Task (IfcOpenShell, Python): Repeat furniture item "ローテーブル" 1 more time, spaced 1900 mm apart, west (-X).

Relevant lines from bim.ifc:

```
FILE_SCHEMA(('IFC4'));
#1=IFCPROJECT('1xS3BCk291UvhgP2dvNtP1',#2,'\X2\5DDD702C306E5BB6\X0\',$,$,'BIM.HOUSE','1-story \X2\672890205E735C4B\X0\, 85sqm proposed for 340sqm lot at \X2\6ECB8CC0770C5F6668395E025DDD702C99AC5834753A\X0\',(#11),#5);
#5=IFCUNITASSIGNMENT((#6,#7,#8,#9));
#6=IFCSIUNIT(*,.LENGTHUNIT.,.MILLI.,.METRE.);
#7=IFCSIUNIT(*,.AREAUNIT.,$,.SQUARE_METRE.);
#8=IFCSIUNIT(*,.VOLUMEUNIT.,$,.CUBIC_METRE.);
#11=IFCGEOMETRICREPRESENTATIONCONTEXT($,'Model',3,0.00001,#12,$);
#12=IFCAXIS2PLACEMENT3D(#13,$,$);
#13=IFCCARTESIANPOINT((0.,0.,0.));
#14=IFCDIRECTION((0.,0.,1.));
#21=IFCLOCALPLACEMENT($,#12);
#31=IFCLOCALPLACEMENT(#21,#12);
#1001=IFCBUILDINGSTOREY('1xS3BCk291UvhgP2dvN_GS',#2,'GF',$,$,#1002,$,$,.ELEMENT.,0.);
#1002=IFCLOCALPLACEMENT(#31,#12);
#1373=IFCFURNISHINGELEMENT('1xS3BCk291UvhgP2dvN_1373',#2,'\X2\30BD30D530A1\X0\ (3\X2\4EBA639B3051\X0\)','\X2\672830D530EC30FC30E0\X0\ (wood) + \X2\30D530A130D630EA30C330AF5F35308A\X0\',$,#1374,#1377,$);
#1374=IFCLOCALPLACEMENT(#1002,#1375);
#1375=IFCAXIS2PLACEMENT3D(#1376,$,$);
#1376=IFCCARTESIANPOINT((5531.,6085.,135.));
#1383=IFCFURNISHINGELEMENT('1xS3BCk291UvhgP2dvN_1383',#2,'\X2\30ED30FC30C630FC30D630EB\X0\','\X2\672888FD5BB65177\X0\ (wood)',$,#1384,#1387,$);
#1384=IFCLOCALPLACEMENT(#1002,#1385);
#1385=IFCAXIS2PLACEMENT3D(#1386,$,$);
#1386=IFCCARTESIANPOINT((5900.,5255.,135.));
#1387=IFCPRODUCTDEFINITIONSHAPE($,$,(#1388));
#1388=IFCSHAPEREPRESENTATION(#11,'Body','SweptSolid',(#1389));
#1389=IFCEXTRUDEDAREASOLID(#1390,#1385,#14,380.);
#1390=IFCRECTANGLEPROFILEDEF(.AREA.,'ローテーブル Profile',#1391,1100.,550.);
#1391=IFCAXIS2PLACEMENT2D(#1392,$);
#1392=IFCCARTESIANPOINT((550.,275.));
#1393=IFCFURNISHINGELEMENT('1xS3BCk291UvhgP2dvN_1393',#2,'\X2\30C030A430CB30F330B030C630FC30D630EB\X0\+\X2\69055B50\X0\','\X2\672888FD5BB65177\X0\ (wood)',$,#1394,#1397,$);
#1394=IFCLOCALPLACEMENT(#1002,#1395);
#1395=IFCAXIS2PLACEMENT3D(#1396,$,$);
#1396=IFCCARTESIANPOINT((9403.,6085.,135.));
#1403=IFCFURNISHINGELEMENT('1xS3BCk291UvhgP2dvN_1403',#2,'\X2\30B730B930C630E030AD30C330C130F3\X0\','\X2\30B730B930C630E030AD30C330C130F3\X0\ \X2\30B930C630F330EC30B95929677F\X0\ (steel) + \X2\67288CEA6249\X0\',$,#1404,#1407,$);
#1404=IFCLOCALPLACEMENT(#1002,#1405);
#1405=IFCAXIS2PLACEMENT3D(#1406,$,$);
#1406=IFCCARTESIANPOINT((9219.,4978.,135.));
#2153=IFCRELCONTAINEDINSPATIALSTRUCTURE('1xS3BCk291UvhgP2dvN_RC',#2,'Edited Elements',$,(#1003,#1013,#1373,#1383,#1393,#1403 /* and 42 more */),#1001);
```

```python
import numpy as np
import ifcopenshell
import ifcopenshell.api.geometry
import ifcopenshell.api.root
import ifcopenshell.util.element
import ifcopenshell.util.placement

model = ifcopenshell.open("bim.ifc")


def reuse_history(source, copy):
    """copy_class also copies each property set's owner history, people and application; keep the originals."""
    for rel in copy.IsDefinedBy:
        if rel.is_a("IfcRelDefinesByProperties") and (history := rel.RelatingPropertyDefinition.OwnerHistory):
            rel.RelatingPropertyDefinition.OwnerHistory = source.OwnerHistory
            ifcopenshell.util.element.remove_deep2(model, history)


source = model.by_guid("1xS3BCk291UvhgP2dvN_1383")
base = ifcopenshell.util.placement.get_local_placement(source.ObjectPlacement)
step = np.array([-1.0, 0.0, 0.0]) * 1900.0

for i in range(1, 2):
    copy = ifcopenshell.api.root.copy_class(model, product=source)
    copy.Representation = ifcopenshell.util.element.copy_deep(
        model, source.Representation, exclude=["IfcGeometricRepresentationContext", "IfcRepresentationMap"]
    )
    reuse_history(source, copy)
    matrix = base.copy()
    matrix[:3, 3] += i * step
    print("added at", matrix[:3, 3].round(3) + 0.0)
    ifcopenshell.api.geometry.edit_object_placement(model, product=copy, matrix=matrix, is_si=False)

model.write("bim_edited.ifc")
```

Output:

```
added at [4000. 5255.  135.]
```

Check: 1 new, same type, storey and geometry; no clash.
